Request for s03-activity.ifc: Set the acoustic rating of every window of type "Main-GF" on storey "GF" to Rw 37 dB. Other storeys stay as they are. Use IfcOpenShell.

First a look at what the model holds.

```python
import ifcopenshell
import ifcopenshell.util.element

model = ifcopenshell.open("s03-activity.ifc")
print(model.schema)
storey = next(s for s in model.by_type("IfcBuildingStorey") if s.Name == "GF")
windows = [e for e in ifcopenshell.util.element.get_decomposition(storey) if e.is_a("IfcWindow")]
seen = {}
for e in windows:
    element_type = ifcopenshell.util.element.get_type(e)
    key = (element_type.Name if element_type != e and element_type else None, ifcopenshell.util.element.get_pset(e, "Pset_WindowCommon", "AcousticRating"))
    seen[key] = seen.get(key, 0) + 1
for (name, value), count in sorted(seen.items(), key=str):
    print(count, "x", name, "|", value)
```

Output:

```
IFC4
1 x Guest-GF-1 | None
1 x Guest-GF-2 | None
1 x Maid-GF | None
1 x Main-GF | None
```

```python
import ifcopenshell
import ifcopenshell.api.pset
import ifcopenshell.util.element

model = ifcopenshell.open("s03-activity.ifc")

storey = next(s for s in model.by_type("IfcBuildingStorey") if s.Name == "GF")
windows = [e for e in ifcopenshell.util.element.get_decomposition(storey) if e.is_a("IfcWindow")]

count = 0
for e in windows:
    element_type = ifcopenshell.util.element.get_type(e)
    if element_type in (None, e) or element_type.Name != "Main-GF":
        continue
    # add_pset returns the element's existing set when there is one.
    pset = ifcopenshell.api.pset.add_pset(model, product=e, name="Pset_WindowCommon")
    ifcopenshell.api.pset.edit_pset(model, pset=pset, properties={"AcousticRating": "Rw 37 dB"})
    count += 1

print(count, "windows updated")

model.write("s03-activity-out.ifc")
```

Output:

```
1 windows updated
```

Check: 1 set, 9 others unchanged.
